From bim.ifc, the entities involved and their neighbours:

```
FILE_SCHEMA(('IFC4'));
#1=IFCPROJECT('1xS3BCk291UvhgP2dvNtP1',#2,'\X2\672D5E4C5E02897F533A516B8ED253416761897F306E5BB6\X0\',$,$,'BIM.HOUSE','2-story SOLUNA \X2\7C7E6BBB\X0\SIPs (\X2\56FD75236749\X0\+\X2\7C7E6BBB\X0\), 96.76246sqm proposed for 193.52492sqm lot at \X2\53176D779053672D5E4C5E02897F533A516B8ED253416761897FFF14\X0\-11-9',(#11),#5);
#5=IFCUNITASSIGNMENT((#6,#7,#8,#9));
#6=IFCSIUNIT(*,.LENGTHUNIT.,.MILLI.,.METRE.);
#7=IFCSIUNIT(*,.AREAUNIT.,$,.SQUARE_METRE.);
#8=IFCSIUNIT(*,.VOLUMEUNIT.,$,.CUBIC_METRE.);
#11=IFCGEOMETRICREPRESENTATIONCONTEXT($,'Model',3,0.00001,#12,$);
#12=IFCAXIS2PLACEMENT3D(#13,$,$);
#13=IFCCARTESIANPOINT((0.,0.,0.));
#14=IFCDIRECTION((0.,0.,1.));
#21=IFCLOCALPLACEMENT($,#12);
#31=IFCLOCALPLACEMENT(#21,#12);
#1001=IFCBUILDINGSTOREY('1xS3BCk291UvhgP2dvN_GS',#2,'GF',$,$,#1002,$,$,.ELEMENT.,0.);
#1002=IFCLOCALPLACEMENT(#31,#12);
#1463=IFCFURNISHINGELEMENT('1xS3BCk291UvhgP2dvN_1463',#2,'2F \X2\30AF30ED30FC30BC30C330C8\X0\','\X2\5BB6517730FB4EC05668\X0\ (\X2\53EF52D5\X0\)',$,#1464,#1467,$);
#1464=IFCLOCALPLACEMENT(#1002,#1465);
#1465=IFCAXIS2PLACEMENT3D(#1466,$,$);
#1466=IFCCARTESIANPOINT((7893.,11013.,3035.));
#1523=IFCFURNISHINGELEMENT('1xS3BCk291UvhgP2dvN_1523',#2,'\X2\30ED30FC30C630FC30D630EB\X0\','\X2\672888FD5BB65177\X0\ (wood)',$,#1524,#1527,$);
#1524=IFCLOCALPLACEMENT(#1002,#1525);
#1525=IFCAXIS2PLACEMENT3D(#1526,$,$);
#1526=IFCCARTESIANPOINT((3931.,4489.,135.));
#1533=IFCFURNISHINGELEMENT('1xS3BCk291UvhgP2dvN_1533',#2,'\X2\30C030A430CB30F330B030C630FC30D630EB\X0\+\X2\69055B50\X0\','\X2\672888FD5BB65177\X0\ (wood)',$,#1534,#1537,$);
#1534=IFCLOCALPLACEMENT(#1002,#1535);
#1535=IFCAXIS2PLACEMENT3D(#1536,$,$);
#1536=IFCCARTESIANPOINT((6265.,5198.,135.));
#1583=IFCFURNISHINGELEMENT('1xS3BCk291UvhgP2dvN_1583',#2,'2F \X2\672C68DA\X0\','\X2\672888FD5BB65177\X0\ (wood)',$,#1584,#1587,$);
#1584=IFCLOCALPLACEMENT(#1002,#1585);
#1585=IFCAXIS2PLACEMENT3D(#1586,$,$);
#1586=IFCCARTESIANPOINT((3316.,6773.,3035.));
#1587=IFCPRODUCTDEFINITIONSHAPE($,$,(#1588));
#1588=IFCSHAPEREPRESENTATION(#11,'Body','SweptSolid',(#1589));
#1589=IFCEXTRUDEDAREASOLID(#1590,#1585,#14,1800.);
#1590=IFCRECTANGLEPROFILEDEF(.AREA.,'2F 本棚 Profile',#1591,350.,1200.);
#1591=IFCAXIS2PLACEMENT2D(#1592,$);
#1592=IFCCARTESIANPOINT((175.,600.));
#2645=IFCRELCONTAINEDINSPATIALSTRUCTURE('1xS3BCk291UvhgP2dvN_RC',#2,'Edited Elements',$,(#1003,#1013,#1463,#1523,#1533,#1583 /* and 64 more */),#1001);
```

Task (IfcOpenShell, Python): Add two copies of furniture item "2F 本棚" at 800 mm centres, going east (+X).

```python
import numpy as np
import ifcopenshell
import ifcopenshell.api.geometry
import ifcopenshell.api.root
import ifcopenshell.util.element
import ifcopenshell.util.placement
import ifcopenshell.util.unit

model = ifcopenshell.open("bim.ifc")
unit_scale = ifcopenshell.util.unit.calculate_unit_scale(model)


def reuse_history(source, copy):
    """copy_class also copies each property set's owner history, people and application; keep the originals."""
    for rel in copy.IsDefinedBy:
        if rel.is_a("IfcRelDefinesByProperties") and (history := rel.RelatingPropertyDefinition.OwnerHistory):
            rel.RelatingPropertyDefinition.OwnerHistory = source.OwnerHistory
            ifcopenshell.util.element.remove_deep2(model, history)


source = model.by_id(1583)
base = ifcopenshell.util.placement.get_local_placement(source.ObjectPlacement)
step = np.array([1.0, 0.0, 0.0]) * 0.8 / unit_scale

for i in range(1, 3):
    copy = ifcopenshell.api.root.copy_class(model, product=source)
    copy.Representation = ifcopenshell.util.element.copy_deep(
        model, source.Representation, exclude=["IfcGeometricRepresentationContext", "IfcRepresentationMap"]
    )
    reuse_history(source, copy)
    matrix = base.copy()
    matrix[:3, 3] += i * step
    print("added at", matrix[:3, 3].round(3) + 0.0)
    ifcopenshell.api.geometry.edit_object_placement(model, product=copy, matrix=matrix, is_si=False)

model.write("bim_edited.ifc")
```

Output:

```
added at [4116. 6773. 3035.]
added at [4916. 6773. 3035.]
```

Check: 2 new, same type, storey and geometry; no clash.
